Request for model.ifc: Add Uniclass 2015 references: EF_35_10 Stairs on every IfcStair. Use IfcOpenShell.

First a look at what the model holds.

```python
import ifcopenshell

model = ifcopenshell.open("model.ifc")
print(model.schema)
print("classifications:", [c.Name for c in model.by_type("IfcClassification")])
for ifc_class in ("IfcDoor", "IfcRoof", "IfcStair", "IfcWall", "IfcWindow"):
    print(ifc_class, len(model.by_type(ifc_class)))
```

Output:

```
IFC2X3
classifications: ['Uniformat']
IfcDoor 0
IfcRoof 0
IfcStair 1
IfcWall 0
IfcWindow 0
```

```python
import ifcopenshell
import ifcopenshell.api.classification

model = ifcopenshell.open("model.ifc")

# IFC2X3 requires Source and Edition and has no link from the project to the system.
system = model.create_entity("IfcClassification", Source="NBS", Edition="2015", Name="Uniclass 2015")

codes = {
    "IfcStair": ("EF_35_10", "Stairs"),
}
for ifc_class, (code, name) in codes.items():
    products = model.by_type(ifc_class)
    ifcopenshell.api.classification.add_reference(
        model, products=products, classification=system, identification=code, name=name
    )
    print(code, len(products))

model.write("model_updated.ifc")
```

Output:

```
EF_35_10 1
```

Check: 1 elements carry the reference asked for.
